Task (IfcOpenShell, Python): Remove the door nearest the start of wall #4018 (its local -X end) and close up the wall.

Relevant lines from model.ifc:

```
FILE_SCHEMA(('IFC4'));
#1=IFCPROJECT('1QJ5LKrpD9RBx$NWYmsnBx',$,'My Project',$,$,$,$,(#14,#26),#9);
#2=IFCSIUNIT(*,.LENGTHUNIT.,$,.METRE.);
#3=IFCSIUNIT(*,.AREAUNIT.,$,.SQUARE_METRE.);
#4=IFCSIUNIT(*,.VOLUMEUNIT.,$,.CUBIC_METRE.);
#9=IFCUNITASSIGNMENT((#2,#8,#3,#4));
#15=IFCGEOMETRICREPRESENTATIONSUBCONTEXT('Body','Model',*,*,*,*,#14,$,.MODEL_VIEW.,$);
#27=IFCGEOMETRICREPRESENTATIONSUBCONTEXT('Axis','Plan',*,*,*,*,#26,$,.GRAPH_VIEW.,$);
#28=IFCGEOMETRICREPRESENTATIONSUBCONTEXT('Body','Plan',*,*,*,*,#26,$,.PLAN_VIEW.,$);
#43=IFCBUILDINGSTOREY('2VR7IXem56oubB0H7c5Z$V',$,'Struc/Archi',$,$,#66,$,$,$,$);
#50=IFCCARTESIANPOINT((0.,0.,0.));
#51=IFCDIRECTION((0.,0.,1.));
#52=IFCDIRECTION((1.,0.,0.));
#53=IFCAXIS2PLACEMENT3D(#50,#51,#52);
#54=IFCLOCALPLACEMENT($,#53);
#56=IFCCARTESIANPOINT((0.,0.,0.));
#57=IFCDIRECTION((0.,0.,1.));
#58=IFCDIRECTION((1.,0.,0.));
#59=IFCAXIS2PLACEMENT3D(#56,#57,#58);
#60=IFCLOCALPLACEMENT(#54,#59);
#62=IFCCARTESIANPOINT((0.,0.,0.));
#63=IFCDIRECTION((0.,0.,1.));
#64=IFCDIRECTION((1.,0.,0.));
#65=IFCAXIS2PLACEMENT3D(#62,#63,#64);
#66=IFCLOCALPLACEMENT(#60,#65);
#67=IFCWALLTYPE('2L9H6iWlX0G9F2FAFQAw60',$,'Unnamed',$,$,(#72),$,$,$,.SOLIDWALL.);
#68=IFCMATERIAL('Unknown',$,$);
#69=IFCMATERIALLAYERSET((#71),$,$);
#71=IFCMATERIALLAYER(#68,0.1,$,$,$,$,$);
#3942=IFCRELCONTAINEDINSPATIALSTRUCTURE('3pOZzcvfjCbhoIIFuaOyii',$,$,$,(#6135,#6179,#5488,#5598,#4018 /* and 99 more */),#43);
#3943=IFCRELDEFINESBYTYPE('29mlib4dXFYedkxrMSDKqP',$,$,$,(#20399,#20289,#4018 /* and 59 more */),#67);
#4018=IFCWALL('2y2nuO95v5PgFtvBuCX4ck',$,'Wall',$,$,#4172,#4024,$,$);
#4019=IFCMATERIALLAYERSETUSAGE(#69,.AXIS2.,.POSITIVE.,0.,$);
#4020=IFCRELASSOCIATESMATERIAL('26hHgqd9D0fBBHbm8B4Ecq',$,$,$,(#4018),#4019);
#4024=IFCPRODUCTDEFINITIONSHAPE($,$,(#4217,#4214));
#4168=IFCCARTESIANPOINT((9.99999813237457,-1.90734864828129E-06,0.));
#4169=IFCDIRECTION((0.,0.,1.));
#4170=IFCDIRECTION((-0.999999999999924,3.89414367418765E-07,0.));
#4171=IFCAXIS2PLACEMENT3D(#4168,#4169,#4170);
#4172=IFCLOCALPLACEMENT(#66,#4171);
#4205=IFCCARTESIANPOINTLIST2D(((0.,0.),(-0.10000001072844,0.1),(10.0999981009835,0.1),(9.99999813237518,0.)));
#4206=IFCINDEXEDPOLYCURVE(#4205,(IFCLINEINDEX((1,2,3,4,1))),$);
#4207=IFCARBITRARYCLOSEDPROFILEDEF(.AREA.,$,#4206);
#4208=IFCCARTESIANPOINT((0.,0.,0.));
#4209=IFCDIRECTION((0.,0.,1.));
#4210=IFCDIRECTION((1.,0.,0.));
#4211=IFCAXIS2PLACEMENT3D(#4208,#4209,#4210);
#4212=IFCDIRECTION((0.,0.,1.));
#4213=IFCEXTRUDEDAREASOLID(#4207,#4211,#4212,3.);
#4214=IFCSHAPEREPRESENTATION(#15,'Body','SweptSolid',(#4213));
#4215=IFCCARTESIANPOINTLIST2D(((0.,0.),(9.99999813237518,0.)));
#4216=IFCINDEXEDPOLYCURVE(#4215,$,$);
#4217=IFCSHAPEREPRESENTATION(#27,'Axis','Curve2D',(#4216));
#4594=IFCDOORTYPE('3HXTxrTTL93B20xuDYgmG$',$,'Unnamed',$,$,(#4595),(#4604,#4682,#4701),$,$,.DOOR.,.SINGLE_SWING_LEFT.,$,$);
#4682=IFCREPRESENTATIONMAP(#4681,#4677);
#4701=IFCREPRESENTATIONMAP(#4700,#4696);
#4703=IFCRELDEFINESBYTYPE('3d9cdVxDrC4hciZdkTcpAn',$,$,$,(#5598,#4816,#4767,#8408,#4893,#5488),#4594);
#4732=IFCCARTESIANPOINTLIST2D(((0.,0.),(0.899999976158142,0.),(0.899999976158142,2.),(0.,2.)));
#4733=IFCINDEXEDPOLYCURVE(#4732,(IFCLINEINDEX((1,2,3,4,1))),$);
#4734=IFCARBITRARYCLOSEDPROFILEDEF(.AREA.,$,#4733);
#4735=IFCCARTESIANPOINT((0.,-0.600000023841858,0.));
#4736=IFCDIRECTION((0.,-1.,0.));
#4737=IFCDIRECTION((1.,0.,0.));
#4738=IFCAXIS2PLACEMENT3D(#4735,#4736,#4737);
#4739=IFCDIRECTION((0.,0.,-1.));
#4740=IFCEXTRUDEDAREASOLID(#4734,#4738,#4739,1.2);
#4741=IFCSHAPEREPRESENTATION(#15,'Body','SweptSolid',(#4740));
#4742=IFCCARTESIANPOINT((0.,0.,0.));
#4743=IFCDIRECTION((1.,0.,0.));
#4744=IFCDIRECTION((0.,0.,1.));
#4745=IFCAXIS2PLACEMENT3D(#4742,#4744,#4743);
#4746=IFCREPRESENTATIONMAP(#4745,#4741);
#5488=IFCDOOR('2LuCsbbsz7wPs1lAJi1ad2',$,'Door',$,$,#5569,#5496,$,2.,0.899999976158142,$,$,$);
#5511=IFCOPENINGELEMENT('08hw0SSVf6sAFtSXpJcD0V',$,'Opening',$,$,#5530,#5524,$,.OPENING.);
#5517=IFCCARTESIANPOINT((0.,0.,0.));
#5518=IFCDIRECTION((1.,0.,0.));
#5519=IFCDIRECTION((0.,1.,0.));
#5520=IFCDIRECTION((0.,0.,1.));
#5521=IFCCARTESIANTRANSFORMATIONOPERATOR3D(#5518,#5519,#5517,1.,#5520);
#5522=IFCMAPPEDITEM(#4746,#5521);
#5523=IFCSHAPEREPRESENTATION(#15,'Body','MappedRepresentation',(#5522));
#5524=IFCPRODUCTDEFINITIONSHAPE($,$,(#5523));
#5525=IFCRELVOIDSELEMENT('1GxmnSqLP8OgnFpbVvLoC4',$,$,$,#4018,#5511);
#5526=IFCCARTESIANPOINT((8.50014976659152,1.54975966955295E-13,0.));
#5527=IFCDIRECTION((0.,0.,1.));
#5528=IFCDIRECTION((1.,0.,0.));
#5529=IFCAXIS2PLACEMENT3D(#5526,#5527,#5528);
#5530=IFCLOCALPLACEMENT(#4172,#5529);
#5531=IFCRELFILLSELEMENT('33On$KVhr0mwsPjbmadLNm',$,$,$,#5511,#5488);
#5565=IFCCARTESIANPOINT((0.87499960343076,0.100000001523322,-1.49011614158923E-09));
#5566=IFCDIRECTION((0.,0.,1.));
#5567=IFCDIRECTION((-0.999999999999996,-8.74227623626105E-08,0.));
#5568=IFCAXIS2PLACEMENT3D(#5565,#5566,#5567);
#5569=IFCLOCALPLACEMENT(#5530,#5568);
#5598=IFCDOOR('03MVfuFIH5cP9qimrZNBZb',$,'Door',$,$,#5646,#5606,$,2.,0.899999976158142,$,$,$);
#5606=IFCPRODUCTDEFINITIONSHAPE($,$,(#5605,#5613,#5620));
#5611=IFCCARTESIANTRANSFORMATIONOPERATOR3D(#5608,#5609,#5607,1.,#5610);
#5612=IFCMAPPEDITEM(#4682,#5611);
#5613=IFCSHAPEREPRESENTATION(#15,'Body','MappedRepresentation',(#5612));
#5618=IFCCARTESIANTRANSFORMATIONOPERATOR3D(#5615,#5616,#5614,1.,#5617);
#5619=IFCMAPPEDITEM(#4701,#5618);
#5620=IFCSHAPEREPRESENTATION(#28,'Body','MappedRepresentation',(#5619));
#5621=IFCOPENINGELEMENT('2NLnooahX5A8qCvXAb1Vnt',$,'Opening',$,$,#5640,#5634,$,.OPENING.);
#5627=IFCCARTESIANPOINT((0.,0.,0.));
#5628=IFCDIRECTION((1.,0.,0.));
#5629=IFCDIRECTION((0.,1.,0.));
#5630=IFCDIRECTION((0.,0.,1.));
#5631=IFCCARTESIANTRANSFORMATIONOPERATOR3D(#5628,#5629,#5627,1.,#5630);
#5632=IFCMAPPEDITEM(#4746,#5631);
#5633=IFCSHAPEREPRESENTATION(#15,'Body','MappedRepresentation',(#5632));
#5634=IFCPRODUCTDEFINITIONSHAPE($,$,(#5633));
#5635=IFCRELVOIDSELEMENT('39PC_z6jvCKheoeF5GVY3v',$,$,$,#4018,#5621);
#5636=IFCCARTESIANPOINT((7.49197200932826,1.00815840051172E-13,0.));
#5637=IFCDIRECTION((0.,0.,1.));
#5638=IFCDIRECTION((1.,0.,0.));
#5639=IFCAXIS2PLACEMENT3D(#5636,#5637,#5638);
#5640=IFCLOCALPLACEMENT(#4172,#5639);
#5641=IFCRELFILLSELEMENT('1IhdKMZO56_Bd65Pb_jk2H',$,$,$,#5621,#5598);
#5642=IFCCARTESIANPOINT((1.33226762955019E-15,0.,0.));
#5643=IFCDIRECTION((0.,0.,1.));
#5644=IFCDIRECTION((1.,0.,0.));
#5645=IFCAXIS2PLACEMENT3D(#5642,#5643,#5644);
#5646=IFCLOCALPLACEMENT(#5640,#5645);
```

```python
import ifcopenshell
import ifcopenshell.api.feature
import ifcopenshell.api.root
import ifcopenshell.geom
import ifcopenshell.util.shape

model = ifcopenshell.open("model.ifc")
settings = ifcopenshell.geom.settings()


def volume(element):
    """Net volume in cubic metres, openings subtracted."""
    shape = ifcopenshell.geom.create_shape(settings, element)
    return ifcopenshell.util.shape.get_volume(shape.geometry)


door = model.by_guid("03MVfuFIH5cP9qimrZNBZb")
opening = door.FillsVoids[0].RelatingOpeningElement
wall = opening.VoidsElements[0].RelatingBuildingElement
before = volume(wall)

ifcopenshell.api.root.remove_product(model, product=door)
ifcopenshell.api.feature.remove_feature(model, feature=opening)

after = volume(wall)

print(f"wall volume {before:.3f} -> {after:.3f} m3")

model.write("model_rev.ifc")
```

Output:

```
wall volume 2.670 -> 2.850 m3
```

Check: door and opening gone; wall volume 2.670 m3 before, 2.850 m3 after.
